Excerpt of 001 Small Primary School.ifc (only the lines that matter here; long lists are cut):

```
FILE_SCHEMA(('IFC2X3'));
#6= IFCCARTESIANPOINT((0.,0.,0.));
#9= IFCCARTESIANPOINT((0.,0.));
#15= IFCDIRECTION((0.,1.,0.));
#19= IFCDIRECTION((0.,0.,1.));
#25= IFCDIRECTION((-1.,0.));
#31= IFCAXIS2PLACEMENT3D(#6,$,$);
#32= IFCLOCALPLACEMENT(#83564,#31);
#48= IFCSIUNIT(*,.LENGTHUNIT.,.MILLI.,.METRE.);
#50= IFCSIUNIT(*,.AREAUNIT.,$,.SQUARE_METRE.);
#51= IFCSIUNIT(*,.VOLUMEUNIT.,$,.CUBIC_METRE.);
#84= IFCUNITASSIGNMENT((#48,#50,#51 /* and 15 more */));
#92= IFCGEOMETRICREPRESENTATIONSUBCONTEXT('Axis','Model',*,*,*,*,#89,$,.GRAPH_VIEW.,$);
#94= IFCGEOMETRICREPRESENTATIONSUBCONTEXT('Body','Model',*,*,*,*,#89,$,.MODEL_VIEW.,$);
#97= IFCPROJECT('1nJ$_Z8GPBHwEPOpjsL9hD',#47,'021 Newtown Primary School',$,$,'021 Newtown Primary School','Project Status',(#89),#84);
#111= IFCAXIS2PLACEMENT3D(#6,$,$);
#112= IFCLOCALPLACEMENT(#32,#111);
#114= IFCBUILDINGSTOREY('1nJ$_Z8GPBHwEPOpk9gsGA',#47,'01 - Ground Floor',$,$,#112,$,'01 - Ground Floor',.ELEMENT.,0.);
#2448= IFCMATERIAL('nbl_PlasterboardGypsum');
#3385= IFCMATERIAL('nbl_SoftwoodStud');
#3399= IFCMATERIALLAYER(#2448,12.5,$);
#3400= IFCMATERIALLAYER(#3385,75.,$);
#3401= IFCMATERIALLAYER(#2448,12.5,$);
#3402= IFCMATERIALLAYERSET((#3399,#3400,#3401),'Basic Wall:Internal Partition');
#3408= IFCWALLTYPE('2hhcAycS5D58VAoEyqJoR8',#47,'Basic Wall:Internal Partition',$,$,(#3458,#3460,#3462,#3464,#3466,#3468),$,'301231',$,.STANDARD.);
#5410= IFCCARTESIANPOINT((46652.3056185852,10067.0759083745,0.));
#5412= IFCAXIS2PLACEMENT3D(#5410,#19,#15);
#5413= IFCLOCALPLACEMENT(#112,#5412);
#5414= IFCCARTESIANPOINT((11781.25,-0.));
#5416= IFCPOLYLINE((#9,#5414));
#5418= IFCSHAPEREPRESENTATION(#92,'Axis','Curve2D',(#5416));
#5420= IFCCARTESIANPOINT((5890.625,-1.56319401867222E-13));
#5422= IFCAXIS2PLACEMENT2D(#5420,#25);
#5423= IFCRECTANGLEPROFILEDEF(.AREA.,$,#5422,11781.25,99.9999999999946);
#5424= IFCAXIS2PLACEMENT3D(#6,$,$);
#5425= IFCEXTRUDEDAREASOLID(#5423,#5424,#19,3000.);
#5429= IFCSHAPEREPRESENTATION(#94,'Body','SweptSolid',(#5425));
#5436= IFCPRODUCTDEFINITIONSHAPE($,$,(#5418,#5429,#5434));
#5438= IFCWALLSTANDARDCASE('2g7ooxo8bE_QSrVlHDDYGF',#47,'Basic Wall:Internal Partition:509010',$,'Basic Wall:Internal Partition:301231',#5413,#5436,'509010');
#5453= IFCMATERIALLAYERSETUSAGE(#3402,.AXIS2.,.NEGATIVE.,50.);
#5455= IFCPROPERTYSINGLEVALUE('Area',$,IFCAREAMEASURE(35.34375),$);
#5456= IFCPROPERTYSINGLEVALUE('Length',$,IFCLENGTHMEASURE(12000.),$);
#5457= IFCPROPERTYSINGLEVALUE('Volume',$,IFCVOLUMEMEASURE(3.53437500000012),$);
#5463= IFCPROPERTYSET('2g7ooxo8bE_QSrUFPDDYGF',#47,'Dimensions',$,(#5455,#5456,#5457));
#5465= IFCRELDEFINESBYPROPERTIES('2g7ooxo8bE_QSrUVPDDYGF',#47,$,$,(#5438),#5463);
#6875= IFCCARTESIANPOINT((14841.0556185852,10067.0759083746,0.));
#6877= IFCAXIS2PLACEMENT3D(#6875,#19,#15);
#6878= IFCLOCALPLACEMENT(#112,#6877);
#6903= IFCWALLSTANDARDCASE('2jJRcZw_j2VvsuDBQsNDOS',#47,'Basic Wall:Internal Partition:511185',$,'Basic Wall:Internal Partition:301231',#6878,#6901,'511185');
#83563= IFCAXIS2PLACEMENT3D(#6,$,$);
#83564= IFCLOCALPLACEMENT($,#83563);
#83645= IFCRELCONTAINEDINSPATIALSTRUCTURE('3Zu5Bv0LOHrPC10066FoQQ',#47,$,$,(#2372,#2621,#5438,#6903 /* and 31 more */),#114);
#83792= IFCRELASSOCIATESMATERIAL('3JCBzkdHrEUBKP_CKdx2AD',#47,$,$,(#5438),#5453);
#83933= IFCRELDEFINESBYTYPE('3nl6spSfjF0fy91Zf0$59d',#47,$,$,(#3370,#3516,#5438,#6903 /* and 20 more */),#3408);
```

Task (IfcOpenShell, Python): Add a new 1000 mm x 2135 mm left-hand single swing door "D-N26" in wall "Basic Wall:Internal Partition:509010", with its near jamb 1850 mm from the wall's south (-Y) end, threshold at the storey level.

```python
import numpy as np
import ifcopenshell
import ifcopenshell.api.feature
import ifcopenshell.api.geometry
import ifcopenshell.api.pset
import ifcopenshell.api.root
import ifcopenshell.api.spatial
import ifcopenshell.api.type
import ifcopenshell.geom
import ifcopenshell.util.element
import ifcopenshell.util.placement
import ifcopenshell.util.representation
import ifcopenshell.util.shape
import ifcopenshell.util.unit

model = ifcopenshell.open("001 Small Primary School.ifc")
unit_scale = ifcopenshell.util.unit.calculate_unit_scale(model)
area_scale = ifcopenshell.util.unit.calculate_unit_scale(model, "AREAUNIT")
volume_scale = ifcopenshell.util.unit.calculate_unit_scale(model, "VOLUMEUNIT")
settings = ifcopenshell.geom.settings()


def volume(element):
    """Net volume in cubic metres, openings subtracted."""
    shape = ifcopenshell.geom.create_shape(settings, element)
    return ifcopenshell.util.shape.get_volume(shape.geometry)


wall = model.by_id(5438)
storey = ifcopenshell.util.element.get_container(wall, ifc_class="IfcBuildingStorey")
context = ifcopenshell.util.representation.get_context(model, "Model", "Body", "MODEL_VIEW")
before = volume(wall)

width, height, from_end, sill = 1, 2.135, 1.85, 0.0  # metres

# The wall runs along its own X axis, and the end named is its -X end.
wall_shape = ifcopenshell.geom.create_shape(settings, wall)
x, y, z = ifcopenshell.util.shape.get_vertices(wall_shape.geometry).T
start = x.min() + from_end
face, thickness = float(y.min()), float(y.max() - y.min())
wall_matrix = ifcopenshell.util.placement.get_local_placement(wall.ObjectPlacement)
level = ifcopenshell.util.placement.get_local_placement(storey.ObjectPlacement)[2, 3]


def in_wall(x, y):
    """Placement at x, y metres in the wall's axes, at sill height."""
    matrix = wall_matrix.copy()
    matrix[:, 3] = wall_matrix @ np.array([x / unit_scale, y / unit_scale, 0.0, 1.0])
    matrix[2, 3] = level + sill / unit_scale
    return matrix


# Opening: a box that overshoots both wall faces by 50 mm.
opening = ifcopenshell.api.root.create_entity(model, ifc_class="IfcOpeningElement")
box = ifcopenshell.api.geometry.add_wall_representation(
    model, context=context, length=width, height=height, thickness=thickness + 0.1
)
ifcopenshell.api.geometry.assign_representation(model, product=opening, representation=box)
ifcopenshell.api.geometry.edit_object_placement(model, product=opening, matrix=in_wall(start, face - 0.05), is_si=False)
ifcopenshell.api.feature.add_feature(model, feature=opening, element=wall)

door = ifcopenshell.api.root.create_entity(model, ifc_class="IfcDoor", name="D-N26")
door.OverallWidth, door.OverallHeight = width / unit_scale, height / unit_scale
body = ifcopenshell.api.geometry.add_door_representation(
    model,
    context=context,
    overall_width=door.OverallWidth,
    overall_height=door.OverallHeight,
    operation_type="SINGLE_SWING_LEFT",
    lining_properties={"LiningDepth": thickness / unit_scale, "ThresholdDepth": thickness / unit_scale},
)
ifcopenshell.api.geometry.assign_representation(model, product=door, representation=body)
ifcopenshell.api.spatial.assign_container(model, products=[door], relating_structure=storey)
fills = ifcopenshell.api.feature.add_filling(model, opening=opening, element=door)
fills.OwnerHistory = door.OwnerHistory  # required in IFC2X3

# IFC2X3 keeps the operation on the door style.
style = ifcopenshell.api.root.create_entity(model, ifc_class="IfcDoorStyle", name="D-N26")
style.OperationType, style.ConstructionType = "SINGLE_SWING_LEFT", "NOTDEFINED"
style.ParameterTakesPrecedence = style.Sizeable = False
ifcopenshell.api.type.assign_type(model, related_objects=[door], relating_type=style)

# The lining spans the wall, so the door starts at the wall face.
ifcopenshell.api.geometry.edit_object_placement(model, product=door, matrix=in_wall(start, face), is_si=False)

after = volume(wall)

# Update the wall's stored quantities.
pset = model.by_id(ifcopenshell.util.element.get_pset(wall, "Dimensions", should_inherit=False)["id"])
ifcopenshell.api.pset.edit_pset(model, pset=pset, properties={
    "Area": model.create_entity("IfcAreaMeasure", after / thickness / area_scale),
    "Volume": model.create_entity("IfcVolumeMeasure", after / volume_scale),
})

print(f"wall volume {before:.3f} -> {after:.3f} m3")

model.write("001 Small Primary School_updated.ifc")
```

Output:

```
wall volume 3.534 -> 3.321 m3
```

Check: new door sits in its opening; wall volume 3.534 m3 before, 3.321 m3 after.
